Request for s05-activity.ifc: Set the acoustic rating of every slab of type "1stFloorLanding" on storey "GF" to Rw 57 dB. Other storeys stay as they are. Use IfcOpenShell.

First a look at what the model holds.

```python
import ifcopenshell
import ifcopenshell.util.element

model = ifcopenshell.open("s05-activity.ifc")
print(model.schema)
storey = next(s for s in model.by_type("IfcBuildingStorey") if s.Name == "GF")
slabs = [e for e in ifcopenshell.util.element.get_decomposition(storey) if e.is_a("IfcSlab")]
seen = {}
for e in slabs:
    element_type = ifcopenshell.util.element.get_type(e)
    key = (element_type.Name if element_type != e and element_type else None, ifcopenshell.util.element.get_pset(e, "Pset_SlabCommon", "AcousticRating"))
    seen[key] = seen.get(key, 0) + 1
for (name, value), count in sorted(seen.items(), key=str):
    print(count, "x", name, "|", value)
```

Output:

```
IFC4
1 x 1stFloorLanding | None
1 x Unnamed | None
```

```python
import ifcopenshell
import ifcopenshell.api.pset
import ifcopenshell.util.element

model = ifcopenshell.open("s05-activity.ifc")

storey = next(s for s in model.by_type("IfcBuildingStorey") if s.Name == "GF")
slabs = [e for e in ifcopenshell.util.element.get_decomposition(storey) if e.is_a("IfcSlab")]

count = 0
for e in slabs:
    element_type = ifcopenshell.util.element.get_type(e)
    if element_type in (None, e) or element_type.Name != "1stFloorLanding":
        continue
    # add_pset returns the element's existing set when there is one.
    pset = ifcopenshell.api.pset.add_pset(model, product=e, name="Pset_SlabCommon")
    ifcopenshell.api.pset.edit_pset(model, pset=pset, properties={"AcousticRating": "Rw 57 dB"})
    count += 1

print(count, "slabs updated")

model.write("s05-activity-out.ifc")
```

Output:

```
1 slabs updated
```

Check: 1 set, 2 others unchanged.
